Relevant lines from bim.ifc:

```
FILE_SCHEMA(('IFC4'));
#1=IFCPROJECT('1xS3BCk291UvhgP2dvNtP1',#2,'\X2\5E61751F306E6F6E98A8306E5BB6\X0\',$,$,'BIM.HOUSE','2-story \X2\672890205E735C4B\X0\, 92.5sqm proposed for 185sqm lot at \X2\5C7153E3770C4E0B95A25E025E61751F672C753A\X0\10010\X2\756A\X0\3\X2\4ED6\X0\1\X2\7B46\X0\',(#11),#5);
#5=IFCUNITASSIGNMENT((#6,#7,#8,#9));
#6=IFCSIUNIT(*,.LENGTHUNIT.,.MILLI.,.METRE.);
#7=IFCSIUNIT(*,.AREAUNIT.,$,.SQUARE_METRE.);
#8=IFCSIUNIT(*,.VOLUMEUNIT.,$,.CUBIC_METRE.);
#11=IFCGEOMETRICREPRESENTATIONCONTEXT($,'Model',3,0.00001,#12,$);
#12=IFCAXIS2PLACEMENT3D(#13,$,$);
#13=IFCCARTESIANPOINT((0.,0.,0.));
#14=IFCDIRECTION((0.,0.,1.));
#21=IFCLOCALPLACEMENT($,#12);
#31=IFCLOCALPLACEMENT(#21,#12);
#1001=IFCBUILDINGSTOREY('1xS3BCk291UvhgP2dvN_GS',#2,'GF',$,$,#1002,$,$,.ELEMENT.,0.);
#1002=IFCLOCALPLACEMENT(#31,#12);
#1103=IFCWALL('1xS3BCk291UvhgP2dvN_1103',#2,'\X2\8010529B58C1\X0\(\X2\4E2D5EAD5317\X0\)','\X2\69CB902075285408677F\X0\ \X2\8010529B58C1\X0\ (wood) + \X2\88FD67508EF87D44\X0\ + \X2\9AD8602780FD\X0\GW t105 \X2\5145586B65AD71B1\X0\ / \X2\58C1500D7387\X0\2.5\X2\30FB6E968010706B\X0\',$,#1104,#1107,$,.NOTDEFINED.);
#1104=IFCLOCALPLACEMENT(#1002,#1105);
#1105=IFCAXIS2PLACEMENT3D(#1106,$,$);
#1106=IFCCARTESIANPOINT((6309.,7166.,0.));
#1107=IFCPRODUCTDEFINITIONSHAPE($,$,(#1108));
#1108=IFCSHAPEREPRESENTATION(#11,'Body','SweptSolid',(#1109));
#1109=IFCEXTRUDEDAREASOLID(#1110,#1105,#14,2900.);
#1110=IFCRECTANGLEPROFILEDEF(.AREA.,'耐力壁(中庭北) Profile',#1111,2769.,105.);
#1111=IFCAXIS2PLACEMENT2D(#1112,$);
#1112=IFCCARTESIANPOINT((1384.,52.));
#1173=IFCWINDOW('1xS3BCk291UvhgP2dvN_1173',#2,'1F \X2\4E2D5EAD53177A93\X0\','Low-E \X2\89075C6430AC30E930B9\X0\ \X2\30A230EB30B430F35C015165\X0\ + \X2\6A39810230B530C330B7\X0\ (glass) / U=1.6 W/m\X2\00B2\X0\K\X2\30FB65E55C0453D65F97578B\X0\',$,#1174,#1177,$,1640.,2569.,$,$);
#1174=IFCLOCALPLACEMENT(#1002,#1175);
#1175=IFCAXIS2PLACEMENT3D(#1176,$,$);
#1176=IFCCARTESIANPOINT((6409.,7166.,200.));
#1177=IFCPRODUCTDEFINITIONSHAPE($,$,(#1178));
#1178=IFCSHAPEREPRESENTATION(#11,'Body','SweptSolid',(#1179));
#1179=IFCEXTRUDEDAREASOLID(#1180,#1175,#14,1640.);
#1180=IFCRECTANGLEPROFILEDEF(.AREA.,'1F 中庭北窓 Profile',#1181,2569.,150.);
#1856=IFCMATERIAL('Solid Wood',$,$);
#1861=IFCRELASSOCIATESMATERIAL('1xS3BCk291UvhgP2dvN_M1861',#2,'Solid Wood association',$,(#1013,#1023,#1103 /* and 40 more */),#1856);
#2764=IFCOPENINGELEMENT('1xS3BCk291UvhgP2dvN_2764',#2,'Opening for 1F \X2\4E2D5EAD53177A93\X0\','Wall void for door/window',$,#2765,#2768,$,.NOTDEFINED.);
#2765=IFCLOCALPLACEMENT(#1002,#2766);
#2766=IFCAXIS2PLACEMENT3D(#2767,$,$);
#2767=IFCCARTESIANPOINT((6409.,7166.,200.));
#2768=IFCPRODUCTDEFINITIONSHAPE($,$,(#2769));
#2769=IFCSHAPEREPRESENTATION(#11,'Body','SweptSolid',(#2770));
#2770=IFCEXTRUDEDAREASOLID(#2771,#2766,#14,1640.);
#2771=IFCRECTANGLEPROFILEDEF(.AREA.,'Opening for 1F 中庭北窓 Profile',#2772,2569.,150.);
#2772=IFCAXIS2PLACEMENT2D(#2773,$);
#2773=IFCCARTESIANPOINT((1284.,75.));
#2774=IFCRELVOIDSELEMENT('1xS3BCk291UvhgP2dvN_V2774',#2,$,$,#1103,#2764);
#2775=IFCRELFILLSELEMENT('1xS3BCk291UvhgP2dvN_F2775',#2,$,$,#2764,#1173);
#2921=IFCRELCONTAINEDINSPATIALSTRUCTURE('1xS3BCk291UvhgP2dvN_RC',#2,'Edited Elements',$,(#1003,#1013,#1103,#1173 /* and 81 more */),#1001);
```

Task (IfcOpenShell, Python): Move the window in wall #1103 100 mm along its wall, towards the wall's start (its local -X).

```python
import ifcopenshell
import ifcopenshell.api.geometry
import ifcopenshell.util.placement
import ifcopenshell.util.unit

model = ifcopenshell.open("bim.ifc")
unit_scale = ifcopenshell.util.unit.calculate_unit_scale(model)

window = model.by_guid("1xS3BCk291UvhgP2dvN_1173")
opening = window.FillsVoids[0].RelatingOpeningElement
wall = opening.VoidsElements[0].RelatingBuildingElement

wall_matrix = ifcopenshell.util.placement.get_local_placement(wall.ObjectPlacement)
shift = wall_matrix[:3, 0] * -0.1 / unit_scale
before = ifcopenshell.util.placement.get_local_placement(window.ObjectPlacement)[:3, 3].copy()

# The window is not placed relative to its opening, so move both.
for product in (opening, window):
    matrix = ifcopenshell.util.placement.get_local_placement(product.ObjectPlacement)
    matrix[:3, 3] += shift
    ifcopenshell.api.geometry.edit_object_placement(model, product=product, matrix=matrix, is_si=False)

after = ifcopenshell.util.placement.get_local_placement(window.ObjectPlacement)[:3, 3]
print("window moved by", (after - before).round(3) + 0.0)

model.write("bim-out.ifc")
```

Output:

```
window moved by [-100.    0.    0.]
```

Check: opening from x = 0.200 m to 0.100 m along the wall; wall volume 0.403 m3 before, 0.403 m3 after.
